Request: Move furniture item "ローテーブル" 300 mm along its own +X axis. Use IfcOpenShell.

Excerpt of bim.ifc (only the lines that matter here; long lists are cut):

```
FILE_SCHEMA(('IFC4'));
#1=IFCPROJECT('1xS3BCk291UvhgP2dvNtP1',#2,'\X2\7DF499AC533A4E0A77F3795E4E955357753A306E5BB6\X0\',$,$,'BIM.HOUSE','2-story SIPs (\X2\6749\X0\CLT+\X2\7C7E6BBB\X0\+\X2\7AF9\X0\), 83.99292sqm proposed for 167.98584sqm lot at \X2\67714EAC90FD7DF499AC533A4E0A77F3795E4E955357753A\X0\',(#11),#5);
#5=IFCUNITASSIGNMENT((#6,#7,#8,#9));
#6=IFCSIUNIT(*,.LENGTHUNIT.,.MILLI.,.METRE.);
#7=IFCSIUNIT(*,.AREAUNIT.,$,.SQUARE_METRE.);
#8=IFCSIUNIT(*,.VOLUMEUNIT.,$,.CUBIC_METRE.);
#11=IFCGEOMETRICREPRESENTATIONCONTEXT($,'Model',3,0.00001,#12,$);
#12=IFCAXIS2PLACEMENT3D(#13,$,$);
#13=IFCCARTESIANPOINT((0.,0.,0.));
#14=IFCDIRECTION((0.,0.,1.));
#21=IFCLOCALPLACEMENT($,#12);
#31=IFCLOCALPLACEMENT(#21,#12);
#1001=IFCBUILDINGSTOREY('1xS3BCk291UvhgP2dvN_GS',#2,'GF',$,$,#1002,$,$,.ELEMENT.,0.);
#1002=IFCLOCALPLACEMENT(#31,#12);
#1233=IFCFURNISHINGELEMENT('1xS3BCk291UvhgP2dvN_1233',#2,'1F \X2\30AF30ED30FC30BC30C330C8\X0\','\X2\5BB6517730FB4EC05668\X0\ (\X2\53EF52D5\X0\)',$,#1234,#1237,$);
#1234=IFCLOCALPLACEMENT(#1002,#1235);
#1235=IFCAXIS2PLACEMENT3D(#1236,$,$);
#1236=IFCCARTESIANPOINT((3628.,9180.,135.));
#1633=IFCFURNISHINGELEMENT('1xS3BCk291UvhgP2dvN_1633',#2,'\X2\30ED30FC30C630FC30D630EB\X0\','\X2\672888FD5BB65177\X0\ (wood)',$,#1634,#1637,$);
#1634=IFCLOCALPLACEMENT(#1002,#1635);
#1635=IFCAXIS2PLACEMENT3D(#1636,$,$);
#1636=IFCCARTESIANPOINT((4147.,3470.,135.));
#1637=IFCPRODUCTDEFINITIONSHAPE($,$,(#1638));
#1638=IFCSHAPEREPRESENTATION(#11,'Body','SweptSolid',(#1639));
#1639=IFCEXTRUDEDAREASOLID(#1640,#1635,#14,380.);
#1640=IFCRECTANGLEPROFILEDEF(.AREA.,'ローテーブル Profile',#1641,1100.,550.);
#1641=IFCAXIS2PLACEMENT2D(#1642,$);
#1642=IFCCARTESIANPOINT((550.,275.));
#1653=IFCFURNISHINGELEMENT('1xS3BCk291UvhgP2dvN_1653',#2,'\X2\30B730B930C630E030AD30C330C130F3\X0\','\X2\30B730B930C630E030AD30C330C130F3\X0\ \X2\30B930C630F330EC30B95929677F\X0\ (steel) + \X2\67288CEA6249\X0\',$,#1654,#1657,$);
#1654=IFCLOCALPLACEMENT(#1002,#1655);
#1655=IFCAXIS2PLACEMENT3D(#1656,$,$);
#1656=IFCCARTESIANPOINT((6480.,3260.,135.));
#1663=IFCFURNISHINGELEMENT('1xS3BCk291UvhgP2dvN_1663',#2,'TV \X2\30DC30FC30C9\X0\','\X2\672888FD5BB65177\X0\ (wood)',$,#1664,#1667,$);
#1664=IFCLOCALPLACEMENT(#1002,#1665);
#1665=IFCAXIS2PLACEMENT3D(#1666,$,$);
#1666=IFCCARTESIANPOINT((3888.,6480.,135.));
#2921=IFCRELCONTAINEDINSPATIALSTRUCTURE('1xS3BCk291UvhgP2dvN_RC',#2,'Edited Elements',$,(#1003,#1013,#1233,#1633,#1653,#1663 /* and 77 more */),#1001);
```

```python
import ifcopenshell
import ifcopenshell.api.geometry
import ifcopenshell.util.placement

model = ifcopenshell.open("bim.ifc")

item = model.by_guid("1xS3BCk291UvhgP2dvN_1633")
matrix = ifcopenshell.util.placement.get_local_placement(item.ObjectPlacement)
matrix[:3, 3] += matrix[:3, 0] * 300.0
ifcopenshell.api.geometry.edit_object_placement(model, product=item, matrix=matrix, is_si=False)

print(ifcopenshell.util.placement.get_local_placement(item.ObjectPlacement).round(3) + 0.0)

model.write("bim-out.ifc")
```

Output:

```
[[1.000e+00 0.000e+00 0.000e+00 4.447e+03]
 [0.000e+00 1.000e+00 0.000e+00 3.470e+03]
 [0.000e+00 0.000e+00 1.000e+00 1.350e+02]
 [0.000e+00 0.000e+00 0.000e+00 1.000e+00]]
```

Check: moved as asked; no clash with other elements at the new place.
